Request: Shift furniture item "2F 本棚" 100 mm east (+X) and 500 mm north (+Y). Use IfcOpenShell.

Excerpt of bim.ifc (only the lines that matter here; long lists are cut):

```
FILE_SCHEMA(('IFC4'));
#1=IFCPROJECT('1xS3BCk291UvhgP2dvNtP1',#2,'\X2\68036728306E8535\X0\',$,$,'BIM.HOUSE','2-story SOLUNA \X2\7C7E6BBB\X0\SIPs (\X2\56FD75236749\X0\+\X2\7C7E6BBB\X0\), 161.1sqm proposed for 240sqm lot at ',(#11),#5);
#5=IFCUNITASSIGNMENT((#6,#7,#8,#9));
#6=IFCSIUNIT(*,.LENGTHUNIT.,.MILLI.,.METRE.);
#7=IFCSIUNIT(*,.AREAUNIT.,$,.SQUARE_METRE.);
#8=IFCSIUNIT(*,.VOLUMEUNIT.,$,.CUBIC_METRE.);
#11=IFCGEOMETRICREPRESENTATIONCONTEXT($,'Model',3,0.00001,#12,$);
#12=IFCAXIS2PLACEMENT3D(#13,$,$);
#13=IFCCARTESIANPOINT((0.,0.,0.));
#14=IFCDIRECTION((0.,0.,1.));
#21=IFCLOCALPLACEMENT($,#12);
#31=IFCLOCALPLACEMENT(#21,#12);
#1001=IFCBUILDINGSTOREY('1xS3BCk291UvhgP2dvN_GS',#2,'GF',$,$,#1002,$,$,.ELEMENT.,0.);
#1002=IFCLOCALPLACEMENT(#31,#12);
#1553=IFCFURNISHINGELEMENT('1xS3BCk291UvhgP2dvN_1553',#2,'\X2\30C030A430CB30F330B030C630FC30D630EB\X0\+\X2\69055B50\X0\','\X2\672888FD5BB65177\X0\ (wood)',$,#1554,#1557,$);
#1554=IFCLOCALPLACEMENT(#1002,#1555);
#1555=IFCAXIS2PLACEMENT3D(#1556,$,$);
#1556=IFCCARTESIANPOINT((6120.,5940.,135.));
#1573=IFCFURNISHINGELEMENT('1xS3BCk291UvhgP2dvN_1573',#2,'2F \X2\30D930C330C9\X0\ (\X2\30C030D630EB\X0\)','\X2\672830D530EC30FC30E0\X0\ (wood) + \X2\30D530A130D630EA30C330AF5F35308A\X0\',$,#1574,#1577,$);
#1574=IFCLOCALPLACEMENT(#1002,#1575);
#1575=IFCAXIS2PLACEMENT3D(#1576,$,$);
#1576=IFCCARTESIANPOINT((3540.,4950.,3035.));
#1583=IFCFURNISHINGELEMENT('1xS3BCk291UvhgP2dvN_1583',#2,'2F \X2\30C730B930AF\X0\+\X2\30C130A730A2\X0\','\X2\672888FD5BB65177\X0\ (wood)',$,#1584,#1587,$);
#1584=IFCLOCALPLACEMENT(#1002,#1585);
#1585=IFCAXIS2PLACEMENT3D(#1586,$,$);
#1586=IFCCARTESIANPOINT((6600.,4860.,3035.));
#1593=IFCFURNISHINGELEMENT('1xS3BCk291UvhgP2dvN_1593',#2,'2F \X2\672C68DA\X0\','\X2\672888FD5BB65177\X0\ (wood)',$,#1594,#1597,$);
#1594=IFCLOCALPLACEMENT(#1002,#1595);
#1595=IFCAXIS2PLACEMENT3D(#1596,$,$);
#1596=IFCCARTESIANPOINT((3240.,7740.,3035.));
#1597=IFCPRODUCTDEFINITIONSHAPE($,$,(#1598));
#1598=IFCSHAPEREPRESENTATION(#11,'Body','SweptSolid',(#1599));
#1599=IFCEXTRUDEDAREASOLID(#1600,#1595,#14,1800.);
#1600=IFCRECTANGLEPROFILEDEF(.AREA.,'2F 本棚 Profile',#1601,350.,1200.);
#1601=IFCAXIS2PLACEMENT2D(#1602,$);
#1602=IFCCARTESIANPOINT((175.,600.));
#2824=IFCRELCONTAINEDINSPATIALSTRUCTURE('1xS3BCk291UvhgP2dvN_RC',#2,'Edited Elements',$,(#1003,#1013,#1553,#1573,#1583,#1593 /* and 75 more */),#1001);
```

```python
import ifcopenshell
import ifcopenshell.api.geometry
import ifcopenshell.util.placement
import ifcopenshell.util.unit

model = ifcopenshell.open("bim.ifc")
unit_scale = ifcopenshell.util.unit.calculate_unit_scale(model)

item = model.by_guid("1xS3BCk291UvhgP2dvN_1593")
matrix = ifcopenshell.util.placement.get_local_placement(item.ObjectPlacement)
matrix[0, 3] += 0.1 / unit_scale
matrix[1, 3] += 0.5 / unit_scale
ifcopenshell.api.geometry.edit_object_placement(model, product=item, matrix=matrix, is_si=False)

print(ifcopenshell.util.placement.get_local_placement(item.ObjectPlacement).round(3) + 0.0)

model.write("bim_updated.ifc")
```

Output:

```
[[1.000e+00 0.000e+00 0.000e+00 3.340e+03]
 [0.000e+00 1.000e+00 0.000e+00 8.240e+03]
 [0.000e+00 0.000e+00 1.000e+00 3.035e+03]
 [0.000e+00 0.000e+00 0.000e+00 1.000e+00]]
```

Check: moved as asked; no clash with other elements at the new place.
